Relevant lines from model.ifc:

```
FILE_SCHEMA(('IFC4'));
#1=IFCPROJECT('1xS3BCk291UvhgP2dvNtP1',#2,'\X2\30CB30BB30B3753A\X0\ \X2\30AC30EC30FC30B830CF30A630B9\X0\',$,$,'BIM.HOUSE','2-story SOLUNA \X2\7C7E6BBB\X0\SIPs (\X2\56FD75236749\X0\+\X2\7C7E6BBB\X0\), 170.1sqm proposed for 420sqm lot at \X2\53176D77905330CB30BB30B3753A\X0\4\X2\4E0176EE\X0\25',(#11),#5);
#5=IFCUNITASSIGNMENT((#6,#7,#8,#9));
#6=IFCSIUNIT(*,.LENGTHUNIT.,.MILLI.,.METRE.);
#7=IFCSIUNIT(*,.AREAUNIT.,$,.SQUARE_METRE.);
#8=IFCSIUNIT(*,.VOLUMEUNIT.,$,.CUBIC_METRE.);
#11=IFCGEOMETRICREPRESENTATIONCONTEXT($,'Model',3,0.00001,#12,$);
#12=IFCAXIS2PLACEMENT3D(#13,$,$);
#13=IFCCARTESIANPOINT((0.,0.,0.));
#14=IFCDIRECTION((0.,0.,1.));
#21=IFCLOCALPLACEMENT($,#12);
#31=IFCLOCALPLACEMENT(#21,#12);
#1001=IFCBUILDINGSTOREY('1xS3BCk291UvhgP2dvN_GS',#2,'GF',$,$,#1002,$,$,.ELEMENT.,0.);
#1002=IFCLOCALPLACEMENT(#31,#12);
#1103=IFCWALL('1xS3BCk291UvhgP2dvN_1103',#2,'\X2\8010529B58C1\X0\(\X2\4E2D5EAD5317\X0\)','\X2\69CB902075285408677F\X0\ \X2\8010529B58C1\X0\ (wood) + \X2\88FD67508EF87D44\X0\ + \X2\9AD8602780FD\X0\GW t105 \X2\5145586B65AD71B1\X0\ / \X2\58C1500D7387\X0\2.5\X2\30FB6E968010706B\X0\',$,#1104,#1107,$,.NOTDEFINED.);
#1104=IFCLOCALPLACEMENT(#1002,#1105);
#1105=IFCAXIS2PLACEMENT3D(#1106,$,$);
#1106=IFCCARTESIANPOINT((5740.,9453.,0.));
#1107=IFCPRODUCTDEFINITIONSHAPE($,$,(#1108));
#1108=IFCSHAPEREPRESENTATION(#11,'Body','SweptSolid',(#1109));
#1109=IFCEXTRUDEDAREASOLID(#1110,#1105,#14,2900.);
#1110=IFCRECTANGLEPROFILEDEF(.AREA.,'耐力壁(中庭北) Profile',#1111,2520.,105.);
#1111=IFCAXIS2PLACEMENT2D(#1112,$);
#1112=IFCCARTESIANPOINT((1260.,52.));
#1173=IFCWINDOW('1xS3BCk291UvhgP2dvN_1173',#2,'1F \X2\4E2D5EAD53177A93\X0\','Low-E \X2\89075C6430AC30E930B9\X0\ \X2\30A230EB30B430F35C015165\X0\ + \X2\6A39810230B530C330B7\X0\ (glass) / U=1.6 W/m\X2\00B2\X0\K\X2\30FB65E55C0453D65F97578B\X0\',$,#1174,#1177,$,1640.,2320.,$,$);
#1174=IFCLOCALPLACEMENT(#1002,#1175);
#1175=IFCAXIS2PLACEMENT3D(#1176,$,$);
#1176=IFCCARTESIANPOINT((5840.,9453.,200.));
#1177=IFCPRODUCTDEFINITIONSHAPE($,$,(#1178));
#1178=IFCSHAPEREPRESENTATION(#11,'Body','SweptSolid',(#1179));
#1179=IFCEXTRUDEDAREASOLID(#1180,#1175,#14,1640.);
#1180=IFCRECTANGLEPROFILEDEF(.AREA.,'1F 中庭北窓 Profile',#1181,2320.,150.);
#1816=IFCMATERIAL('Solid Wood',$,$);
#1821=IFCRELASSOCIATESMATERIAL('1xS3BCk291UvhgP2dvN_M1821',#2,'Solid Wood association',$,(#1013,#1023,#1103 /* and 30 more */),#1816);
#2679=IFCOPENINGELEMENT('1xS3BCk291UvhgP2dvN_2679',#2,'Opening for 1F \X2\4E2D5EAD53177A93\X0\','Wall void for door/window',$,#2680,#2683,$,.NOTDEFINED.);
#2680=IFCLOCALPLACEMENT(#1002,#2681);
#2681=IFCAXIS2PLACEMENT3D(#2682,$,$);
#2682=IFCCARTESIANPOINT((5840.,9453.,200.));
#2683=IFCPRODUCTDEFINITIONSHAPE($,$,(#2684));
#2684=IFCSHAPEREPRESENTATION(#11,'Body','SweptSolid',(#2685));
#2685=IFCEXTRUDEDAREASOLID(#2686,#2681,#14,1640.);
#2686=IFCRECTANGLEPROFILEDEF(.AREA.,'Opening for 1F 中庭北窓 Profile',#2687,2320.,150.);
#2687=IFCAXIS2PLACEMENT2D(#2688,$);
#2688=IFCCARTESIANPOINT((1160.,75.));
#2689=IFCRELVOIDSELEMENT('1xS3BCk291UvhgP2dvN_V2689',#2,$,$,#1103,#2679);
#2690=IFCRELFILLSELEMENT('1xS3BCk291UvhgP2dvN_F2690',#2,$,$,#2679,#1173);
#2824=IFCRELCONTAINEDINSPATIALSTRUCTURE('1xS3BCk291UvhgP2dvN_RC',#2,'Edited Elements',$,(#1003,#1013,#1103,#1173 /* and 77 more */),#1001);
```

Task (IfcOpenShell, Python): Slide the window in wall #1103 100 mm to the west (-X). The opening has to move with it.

```python
import ifcopenshell
import ifcopenshell.api.geometry
import ifcopenshell.util.placement

model = ifcopenshell.open("model.ifc")

window = model.by_guid("1xS3BCk291UvhgP2dvN_1173")
opening = window.FillsVoids[0].RelatingOpeningElement
wall = opening.VoidsElements[0].RelatingBuildingElement

wall_matrix = ifcopenshell.util.placement.get_local_placement(wall.ObjectPlacement)
shift = wall_matrix[:3, 0] * -100.0
before = ifcopenshell.util.placement.get_local_placement(window.ObjectPlacement)[:3, 3].copy()

# The window is not placed relative to its opening, so move both.
for product in (opening, window):
    matrix = ifcopenshell.util.placement.get_local_placement(product.ObjectPlacement)
    matrix[:3, 3] += shift
    ifcopenshell.api.geometry.edit_object_placement(model, product=product, matrix=matrix, is_si=False)

after = ifcopenshell.util.placement.get_local_placement(window.ObjectPlacement)[:3, 3]
print("window moved by", (after - before).round(3) + 0.0)

model.write("model-out.ifc")
```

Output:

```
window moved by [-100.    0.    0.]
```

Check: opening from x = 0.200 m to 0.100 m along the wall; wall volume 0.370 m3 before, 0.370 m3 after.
